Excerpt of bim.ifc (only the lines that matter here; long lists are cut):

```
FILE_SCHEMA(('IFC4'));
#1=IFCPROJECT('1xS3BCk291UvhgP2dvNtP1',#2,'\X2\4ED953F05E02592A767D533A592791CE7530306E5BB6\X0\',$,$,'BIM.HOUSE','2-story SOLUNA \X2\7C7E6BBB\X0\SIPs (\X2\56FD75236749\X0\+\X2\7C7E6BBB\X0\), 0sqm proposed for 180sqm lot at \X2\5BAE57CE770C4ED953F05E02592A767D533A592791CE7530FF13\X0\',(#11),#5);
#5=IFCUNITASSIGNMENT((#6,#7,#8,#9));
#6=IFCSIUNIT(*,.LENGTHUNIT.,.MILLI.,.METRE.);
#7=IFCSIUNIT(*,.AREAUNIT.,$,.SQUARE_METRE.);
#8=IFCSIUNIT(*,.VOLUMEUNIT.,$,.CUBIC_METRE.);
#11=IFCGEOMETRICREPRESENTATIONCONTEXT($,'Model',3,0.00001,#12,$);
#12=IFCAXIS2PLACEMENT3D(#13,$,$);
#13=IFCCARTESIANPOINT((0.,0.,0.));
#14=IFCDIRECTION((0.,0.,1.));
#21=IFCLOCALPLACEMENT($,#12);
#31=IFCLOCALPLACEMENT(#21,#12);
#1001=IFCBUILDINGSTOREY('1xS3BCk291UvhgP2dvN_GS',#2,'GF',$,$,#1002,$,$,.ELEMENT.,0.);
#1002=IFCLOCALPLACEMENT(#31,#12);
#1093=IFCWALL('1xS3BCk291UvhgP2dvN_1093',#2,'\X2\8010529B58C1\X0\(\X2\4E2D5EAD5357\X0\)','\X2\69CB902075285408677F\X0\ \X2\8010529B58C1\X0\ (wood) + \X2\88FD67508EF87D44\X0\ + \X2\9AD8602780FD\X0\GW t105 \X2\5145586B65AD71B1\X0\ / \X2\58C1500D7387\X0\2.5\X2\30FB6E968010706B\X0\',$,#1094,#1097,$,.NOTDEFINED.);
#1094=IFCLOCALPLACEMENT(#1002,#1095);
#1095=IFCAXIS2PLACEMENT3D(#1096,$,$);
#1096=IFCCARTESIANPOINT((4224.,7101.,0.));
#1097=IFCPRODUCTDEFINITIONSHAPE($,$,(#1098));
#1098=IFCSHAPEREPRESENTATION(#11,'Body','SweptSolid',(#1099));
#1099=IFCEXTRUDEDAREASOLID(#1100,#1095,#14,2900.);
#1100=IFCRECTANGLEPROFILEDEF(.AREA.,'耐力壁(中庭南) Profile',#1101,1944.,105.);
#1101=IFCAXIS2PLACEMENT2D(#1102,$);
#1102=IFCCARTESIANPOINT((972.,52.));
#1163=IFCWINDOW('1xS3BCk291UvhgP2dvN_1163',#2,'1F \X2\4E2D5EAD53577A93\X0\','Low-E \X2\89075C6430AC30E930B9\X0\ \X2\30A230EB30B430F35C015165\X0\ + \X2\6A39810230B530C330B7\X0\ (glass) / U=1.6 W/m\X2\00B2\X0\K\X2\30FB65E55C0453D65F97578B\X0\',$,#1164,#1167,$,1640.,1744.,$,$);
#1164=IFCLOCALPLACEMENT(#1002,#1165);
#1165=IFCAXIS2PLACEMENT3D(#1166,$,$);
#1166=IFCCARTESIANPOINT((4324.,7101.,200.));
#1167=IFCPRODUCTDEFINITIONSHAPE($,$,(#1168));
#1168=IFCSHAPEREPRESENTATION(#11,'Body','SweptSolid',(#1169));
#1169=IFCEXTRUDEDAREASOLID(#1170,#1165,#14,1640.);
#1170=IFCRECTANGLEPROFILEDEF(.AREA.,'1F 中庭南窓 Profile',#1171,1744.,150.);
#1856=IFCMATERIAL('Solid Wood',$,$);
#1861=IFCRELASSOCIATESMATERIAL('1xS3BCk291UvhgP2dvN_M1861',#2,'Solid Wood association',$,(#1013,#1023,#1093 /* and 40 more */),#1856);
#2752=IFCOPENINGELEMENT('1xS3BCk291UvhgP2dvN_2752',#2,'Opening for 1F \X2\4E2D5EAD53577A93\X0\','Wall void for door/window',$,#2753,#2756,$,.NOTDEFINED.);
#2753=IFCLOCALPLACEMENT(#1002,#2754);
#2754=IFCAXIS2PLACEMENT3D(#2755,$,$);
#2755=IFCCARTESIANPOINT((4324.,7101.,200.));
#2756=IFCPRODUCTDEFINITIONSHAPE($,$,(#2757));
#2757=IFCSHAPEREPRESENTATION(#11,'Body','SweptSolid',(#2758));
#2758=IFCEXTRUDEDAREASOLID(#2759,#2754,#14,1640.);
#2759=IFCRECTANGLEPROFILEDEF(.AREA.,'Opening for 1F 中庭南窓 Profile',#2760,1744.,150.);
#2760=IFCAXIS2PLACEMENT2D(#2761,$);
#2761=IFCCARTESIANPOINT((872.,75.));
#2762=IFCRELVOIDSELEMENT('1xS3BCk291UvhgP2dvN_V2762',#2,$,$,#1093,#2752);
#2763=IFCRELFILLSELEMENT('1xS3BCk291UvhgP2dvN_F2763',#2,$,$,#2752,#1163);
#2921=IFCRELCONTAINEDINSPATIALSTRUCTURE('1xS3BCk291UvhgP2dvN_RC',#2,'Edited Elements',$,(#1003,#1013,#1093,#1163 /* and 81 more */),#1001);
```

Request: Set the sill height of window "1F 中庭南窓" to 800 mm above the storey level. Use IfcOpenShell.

```python
import numpy as np
import ifcopenshell
import ifcopenshell.api.geometry
import ifcopenshell.geom
import ifcopenshell.util.element
import ifcopenshell.util.placement
import ifcopenshell.util.shape
import ifcopenshell.util.unit

model = ifcopenshell.open("bim.ifc")
unit_scale = ifcopenshell.util.unit.calculate_unit_scale(model)

window = model.by_guid("1xS3BCk291UvhgP2dvN_1163")
opening = window.FillsVoids[0].RelatingOpeningElement
storey = ifcopenshell.util.element.get_container(window, ifc_class="IfcBuildingStorey")
level = ifcopenshell.util.placement.get_local_placement(storey.ObjectPlacement)[2, 3]

# The opening's origin need not be at the sill, so measure its lowest point.
shape = ifcopenshell.geom.create_shape(ifcopenshell.geom.settings(), opening)
bottom = ifcopenshell.util.shape.get_shape_bottom_elevation(shape, shape.geometry) / unit_scale
dz = level + 0.8 / unit_scale - bottom

shift = np.array([0.0, 0.0, dz])
# The window is not placed relative to its opening, so move both.
for product in (opening, window):
    matrix = ifcopenshell.util.placement.get_local_placement(product.ObjectPlacement)
    matrix[:3, 3] += shift
    ifcopenshell.api.geometry.edit_object_placement(model, product=product, matrix=matrix, is_si=False)

print(f"moved by {dz * unit_scale:+.3f} m")

model.write("bim_updated.ifc")
```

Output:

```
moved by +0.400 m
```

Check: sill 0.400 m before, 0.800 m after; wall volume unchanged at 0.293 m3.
